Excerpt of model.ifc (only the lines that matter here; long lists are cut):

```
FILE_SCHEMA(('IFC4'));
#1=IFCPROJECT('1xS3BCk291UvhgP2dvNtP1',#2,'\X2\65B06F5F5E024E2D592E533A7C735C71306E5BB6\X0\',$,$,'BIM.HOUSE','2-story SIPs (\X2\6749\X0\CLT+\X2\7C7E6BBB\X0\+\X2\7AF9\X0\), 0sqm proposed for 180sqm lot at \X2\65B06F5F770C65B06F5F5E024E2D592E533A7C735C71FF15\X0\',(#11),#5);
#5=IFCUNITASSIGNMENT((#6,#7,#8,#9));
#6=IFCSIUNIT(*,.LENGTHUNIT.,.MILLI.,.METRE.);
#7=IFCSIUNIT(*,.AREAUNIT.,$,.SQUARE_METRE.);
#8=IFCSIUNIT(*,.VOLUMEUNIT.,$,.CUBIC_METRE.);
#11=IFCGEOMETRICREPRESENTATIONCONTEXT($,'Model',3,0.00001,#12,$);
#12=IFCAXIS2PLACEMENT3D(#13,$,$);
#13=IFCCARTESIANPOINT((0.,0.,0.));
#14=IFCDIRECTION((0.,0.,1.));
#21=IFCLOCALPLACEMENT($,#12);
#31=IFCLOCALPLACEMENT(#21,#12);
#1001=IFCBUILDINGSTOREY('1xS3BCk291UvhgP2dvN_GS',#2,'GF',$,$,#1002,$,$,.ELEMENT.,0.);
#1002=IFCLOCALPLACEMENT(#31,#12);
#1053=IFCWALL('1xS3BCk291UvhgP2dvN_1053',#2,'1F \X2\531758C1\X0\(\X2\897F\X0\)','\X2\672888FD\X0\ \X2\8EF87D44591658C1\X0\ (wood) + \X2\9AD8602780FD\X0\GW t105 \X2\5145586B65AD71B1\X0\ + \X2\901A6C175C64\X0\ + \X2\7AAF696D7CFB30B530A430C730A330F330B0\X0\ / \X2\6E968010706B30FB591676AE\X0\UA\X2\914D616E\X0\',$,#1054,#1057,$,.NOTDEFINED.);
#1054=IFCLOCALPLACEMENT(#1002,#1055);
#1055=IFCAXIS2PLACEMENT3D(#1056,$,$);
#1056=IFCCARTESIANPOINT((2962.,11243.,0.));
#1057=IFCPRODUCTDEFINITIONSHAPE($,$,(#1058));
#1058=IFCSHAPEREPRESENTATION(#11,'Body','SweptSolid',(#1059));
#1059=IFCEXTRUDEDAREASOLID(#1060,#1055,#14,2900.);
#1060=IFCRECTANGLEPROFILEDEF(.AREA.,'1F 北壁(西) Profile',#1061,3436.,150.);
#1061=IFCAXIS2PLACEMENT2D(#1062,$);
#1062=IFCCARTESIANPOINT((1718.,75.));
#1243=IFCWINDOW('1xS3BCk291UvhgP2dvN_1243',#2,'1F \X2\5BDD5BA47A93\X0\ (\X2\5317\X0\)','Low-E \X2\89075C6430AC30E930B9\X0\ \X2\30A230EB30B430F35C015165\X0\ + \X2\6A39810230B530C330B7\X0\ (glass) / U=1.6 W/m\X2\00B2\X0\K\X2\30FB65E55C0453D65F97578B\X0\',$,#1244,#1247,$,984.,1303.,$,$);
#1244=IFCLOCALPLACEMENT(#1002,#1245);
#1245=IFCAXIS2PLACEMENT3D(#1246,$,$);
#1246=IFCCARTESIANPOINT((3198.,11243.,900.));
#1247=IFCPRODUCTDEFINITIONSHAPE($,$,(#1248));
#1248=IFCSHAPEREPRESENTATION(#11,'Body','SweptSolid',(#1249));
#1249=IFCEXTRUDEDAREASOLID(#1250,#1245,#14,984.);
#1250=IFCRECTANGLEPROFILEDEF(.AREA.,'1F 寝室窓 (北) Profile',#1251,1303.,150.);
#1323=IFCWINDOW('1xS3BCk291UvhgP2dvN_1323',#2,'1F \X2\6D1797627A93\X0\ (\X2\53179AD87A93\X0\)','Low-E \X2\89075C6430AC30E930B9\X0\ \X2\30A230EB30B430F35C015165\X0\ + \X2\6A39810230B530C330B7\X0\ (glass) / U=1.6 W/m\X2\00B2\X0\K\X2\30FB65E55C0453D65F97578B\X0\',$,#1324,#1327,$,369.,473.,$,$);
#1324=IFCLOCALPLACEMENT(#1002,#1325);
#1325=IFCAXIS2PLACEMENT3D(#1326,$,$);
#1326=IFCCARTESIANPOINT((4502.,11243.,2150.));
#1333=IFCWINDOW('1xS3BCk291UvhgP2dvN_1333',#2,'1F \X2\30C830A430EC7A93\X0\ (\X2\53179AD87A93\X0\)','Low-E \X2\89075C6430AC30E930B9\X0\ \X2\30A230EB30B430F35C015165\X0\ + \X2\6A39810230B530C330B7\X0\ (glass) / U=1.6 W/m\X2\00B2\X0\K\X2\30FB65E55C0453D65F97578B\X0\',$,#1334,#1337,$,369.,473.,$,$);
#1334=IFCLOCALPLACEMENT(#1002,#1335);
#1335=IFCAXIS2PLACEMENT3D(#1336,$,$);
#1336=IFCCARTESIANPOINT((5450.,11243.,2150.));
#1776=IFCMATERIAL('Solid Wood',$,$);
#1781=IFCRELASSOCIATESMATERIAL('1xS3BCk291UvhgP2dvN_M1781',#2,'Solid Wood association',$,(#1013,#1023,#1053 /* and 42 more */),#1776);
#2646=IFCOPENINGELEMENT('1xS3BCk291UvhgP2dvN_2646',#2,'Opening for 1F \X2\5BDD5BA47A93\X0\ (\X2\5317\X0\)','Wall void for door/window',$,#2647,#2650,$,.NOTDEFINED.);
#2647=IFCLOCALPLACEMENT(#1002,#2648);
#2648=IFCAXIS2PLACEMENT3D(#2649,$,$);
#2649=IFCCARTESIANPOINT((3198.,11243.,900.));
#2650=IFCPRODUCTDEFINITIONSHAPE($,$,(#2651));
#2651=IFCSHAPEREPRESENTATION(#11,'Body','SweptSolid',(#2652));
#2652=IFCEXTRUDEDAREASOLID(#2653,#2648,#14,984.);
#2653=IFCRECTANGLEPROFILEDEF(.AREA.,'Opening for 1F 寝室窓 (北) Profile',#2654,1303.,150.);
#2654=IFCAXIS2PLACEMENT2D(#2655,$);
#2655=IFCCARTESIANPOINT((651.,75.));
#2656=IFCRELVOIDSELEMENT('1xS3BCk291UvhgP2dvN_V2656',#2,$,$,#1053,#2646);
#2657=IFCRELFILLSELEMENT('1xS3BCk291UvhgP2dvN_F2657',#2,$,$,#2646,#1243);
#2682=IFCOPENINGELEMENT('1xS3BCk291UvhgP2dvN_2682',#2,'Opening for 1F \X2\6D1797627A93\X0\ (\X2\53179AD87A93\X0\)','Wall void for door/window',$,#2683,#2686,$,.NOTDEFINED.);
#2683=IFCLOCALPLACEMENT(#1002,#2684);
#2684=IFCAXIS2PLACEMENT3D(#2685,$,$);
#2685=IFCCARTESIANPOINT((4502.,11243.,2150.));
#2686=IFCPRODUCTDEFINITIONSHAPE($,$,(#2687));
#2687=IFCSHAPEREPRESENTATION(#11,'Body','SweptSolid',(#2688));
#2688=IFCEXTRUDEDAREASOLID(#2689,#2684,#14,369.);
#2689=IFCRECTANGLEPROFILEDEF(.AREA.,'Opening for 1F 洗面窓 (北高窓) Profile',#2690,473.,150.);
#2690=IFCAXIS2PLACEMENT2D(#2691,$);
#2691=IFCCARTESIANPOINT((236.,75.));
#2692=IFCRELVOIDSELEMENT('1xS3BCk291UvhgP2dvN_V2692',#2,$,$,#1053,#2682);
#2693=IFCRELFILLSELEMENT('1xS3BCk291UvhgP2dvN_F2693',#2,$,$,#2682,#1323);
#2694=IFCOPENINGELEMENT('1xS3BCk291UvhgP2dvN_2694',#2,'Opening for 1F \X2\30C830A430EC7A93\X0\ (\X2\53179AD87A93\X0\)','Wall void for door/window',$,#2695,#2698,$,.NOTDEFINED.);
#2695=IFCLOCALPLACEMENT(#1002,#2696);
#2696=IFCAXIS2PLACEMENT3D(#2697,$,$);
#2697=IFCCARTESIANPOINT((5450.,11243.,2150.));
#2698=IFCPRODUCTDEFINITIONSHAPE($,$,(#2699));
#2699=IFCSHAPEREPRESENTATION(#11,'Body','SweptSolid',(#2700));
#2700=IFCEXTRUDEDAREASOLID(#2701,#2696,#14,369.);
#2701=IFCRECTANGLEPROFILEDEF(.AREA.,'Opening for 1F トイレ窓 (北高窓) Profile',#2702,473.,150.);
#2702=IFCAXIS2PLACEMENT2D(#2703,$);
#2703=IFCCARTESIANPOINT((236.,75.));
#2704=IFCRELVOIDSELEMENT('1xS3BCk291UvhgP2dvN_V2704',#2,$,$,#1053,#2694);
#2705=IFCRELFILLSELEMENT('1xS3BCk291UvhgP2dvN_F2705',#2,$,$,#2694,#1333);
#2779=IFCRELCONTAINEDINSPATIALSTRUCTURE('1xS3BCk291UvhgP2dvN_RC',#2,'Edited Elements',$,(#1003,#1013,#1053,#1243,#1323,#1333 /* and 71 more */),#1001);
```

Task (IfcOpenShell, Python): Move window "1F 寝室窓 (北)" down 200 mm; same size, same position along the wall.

```python
import numpy as np
import ifcopenshell
import ifcopenshell.api.geometry
import ifcopenshell.util.placement
import ifcopenshell.util.unit

model = ifcopenshell.open("model.ifc")
unit_scale = ifcopenshell.util.unit.calculate_unit_scale(model)

window = model.by_guid("1xS3BCk291UvhgP2dvN_1243")
opening = window.FillsVoids[0].RelatingOpeningElement
dz = -0.2 / unit_scale

shift = np.array([0.0, 0.0, dz])
# The window is not placed relative to its opening, so move both.
for product in (opening, window):
    matrix = ifcopenshell.util.placement.get_local_placement(product.ObjectPlacement)
    matrix[:3, 3] += shift
    ifcopenshell.api.geometry.edit_object_placement(model, product=product, matrix=matrix, is_si=False)

print(f"moved by {dz * unit_scale:+.3f} m")

model.write("model_v2.ifc")
```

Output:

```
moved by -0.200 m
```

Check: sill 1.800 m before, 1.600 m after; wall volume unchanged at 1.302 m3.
